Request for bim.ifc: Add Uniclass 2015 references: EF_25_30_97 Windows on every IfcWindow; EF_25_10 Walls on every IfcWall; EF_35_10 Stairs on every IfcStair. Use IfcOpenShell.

First a look at what the model holds.

```python
import ifcopenshell

model = ifcopenshell.open("bim.ifc")
print(model.schema)
print("classifications:", [c.Name for c in model.by_type("IfcClassification")])
for ifc_class in ("IfcDoor", "IfcRoof", "IfcStair", "IfcWall", "IfcWindow"):
    print(ifc_class, len(model.by_type(ifc_class)))
```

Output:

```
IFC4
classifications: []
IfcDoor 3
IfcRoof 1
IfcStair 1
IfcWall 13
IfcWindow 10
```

```python
import ifcopenshell
import ifcopenshell.api.classification

model = ifcopenshell.open("bim.ifc")

system = ifcopenshell.api.classification.add_classification(model, classification="Uniclass 2015")

codes = {
    "IfcWindow": ("EF_25_30_97", "Windows"),
    "IfcWall": ("EF_25_10", "Walls"),
    "IfcStair": ("EF_35_10", "Stairs"),
}
for ifc_class, (code, name) in codes.items():
    products = model.by_type(ifc_class)
    ifcopenshell.api.classification.add_reference(
        model, products=products, classification=system, identification=code, name=name
    )
    print(code, len(products))

model.write("bim_edited.ifc")
```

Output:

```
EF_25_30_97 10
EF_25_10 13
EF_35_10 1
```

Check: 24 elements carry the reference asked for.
